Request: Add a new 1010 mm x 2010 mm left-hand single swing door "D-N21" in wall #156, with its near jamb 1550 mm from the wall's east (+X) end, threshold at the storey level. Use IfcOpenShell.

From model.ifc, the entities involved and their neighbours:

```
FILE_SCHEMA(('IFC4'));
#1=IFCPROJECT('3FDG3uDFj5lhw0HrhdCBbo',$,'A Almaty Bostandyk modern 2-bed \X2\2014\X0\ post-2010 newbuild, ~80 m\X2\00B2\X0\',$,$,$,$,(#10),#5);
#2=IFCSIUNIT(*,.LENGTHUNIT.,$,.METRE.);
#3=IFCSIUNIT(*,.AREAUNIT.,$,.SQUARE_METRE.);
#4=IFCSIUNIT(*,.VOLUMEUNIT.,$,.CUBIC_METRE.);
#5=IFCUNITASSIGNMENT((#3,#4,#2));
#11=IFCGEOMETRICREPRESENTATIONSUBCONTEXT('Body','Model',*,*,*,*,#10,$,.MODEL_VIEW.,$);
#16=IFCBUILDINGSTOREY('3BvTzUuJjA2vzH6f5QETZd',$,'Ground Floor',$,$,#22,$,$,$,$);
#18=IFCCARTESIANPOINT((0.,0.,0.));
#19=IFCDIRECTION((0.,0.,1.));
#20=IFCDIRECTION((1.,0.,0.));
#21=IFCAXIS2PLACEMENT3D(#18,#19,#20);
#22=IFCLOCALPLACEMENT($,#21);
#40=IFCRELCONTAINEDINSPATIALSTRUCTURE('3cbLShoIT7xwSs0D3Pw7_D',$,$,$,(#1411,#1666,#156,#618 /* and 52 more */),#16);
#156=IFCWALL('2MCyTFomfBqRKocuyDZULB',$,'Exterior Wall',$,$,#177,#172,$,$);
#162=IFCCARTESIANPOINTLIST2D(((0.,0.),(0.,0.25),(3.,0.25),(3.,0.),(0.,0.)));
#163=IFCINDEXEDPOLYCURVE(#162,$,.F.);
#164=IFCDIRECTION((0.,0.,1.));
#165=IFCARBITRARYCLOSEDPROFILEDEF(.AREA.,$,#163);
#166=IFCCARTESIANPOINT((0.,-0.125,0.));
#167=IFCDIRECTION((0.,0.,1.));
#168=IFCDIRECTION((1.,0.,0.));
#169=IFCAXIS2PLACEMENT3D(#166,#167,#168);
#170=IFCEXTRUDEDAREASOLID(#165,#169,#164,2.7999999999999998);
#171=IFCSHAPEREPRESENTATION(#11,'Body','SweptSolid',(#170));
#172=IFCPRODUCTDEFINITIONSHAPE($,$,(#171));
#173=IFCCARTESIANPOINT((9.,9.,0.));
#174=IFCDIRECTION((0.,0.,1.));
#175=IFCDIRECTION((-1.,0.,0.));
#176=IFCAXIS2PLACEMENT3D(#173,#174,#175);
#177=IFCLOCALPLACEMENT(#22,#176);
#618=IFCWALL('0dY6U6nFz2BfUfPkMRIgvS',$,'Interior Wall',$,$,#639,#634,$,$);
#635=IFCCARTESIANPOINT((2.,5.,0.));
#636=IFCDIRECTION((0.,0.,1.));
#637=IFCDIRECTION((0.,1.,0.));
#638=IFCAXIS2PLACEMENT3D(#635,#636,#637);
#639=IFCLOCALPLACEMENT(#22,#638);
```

```python
import numpy as np
import ifcopenshell
import ifcopenshell.api.feature
import ifcopenshell.api.geometry
import ifcopenshell.api.root
import ifcopenshell.api.spatial
import ifcopenshell.geom
import ifcopenshell.util.element
import ifcopenshell.util.placement
import ifcopenshell.util.representation
import ifcopenshell.util.shape
import ifcopenshell.util.unit

model = ifcopenshell.open("model.ifc")
unit_scale = ifcopenshell.util.unit.calculate_unit_scale(model)
settings = ifcopenshell.geom.settings()


def volume(element):
    """Net volume in cubic metres, openings subtracted."""
    shape = ifcopenshell.geom.create_shape(settings, element)
    return ifcopenshell.util.shape.get_volume(shape.geometry)


wall = model.by_guid("2MCyTFomfBqRKocuyDZULB")
storey = ifcopenshell.util.element.get_container(wall, ifc_class="IfcBuildingStorey")
context = ifcopenshell.util.representation.get_context(model, "Model", "Body", "MODEL_VIEW")
before = volume(wall)

width, height, from_end, sill = 1.01, 2.01, 1.55, 0.0  # metres

# The wall runs along its own X axis, and the end named is its -X end.
wall_shape = ifcopenshell.geom.create_shape(settings, wall)
x, y, z = ifcopenshell.util.shape.get_vertices(wall_shape.geometry).T
start = x.min() + from_end
face, thickness = float(y.min()), float(y.max() - y.min())
wall_matrix = ifcopenshell.util.placement.get_local_placement(wall.ObjectPlacement)
level = ifcopenshell.util.placement.get_local_placement(storey.ObjectPlacement)[2, 3]


def in_wall(x, y):
    """Placement at x, y metres in the wall's axes, at sill height."""
    matrix = wall_matrix.copy()
    matrix[:, 3] = wall_matrix @ np.array([x / unit_scale, y / unit_scale, 0.0, 1.0])
    matrix[2, 3] = level + sill / unit_scale
    return matrix


# Opening: a box that overshoots both wall faces by 50 mm.
opening = ifcopenshell.api.root.create_entity(model, ifc_class="IfcOpeningElement", predefined_type="OPENING")
box = ifcopenshell.api.geometry.add_wall_representation(
    model, context=context, length=width, height=height, thickness=thickness + 0.1
)
ifcopenshell.api.geometry.assign_representation(model, product=opening, representation=box)
ifcopenshell.api.geometry.edit_object_placement(model, product=opening, matrix=in_wall(start, face - 0.05), is_si=False)
ifcopenshell.api.feature.add_feature(model, feature=opening, element=wall)

door = ifcopenshell.api.root.create_entity(model, ifc_class="IfcDoor", name="D-N21", predefined_type="DOOR")
door.OverallWidth, door.OverallHeight = width / unit_scale, height / unit_scale
door.OperationType = "SINGLE_SWING_LEFT"
body = ifcopenshell.api.geometry.add_door_representation(
    model,
    context=context,
    overall_width=door.OverallWidth,
    overall_height=door.OverallHeight,
    operation_type="SINGLE_SWING_LEFT",
    lining_properties={"LiningDepth": thickness / unit_scale, "ThresholdDepth": thickness / unit_scale},
)
ifcopenshell.api.geometry.assign_representation(model, product=door, representation=body)
ifcopenshell.api.spatial.assign_container(model, products=[door], relating_structure=storey)
ifcopenshell.api.feature.add_filling(model, opening=opening, element=door)

# The lining spans the wall, so the door starts at the wall face.
ifcopenshell.api.geometry.edit_object_placement(model, product=door, matrix=in_wall(start, face), is_si=False)

after = volume(wall)

print(f"wall volume {before:.3f} -> {after:.3f} m3")

model.write("model-out.ifc")
```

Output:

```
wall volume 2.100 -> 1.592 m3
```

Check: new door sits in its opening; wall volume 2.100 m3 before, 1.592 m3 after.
